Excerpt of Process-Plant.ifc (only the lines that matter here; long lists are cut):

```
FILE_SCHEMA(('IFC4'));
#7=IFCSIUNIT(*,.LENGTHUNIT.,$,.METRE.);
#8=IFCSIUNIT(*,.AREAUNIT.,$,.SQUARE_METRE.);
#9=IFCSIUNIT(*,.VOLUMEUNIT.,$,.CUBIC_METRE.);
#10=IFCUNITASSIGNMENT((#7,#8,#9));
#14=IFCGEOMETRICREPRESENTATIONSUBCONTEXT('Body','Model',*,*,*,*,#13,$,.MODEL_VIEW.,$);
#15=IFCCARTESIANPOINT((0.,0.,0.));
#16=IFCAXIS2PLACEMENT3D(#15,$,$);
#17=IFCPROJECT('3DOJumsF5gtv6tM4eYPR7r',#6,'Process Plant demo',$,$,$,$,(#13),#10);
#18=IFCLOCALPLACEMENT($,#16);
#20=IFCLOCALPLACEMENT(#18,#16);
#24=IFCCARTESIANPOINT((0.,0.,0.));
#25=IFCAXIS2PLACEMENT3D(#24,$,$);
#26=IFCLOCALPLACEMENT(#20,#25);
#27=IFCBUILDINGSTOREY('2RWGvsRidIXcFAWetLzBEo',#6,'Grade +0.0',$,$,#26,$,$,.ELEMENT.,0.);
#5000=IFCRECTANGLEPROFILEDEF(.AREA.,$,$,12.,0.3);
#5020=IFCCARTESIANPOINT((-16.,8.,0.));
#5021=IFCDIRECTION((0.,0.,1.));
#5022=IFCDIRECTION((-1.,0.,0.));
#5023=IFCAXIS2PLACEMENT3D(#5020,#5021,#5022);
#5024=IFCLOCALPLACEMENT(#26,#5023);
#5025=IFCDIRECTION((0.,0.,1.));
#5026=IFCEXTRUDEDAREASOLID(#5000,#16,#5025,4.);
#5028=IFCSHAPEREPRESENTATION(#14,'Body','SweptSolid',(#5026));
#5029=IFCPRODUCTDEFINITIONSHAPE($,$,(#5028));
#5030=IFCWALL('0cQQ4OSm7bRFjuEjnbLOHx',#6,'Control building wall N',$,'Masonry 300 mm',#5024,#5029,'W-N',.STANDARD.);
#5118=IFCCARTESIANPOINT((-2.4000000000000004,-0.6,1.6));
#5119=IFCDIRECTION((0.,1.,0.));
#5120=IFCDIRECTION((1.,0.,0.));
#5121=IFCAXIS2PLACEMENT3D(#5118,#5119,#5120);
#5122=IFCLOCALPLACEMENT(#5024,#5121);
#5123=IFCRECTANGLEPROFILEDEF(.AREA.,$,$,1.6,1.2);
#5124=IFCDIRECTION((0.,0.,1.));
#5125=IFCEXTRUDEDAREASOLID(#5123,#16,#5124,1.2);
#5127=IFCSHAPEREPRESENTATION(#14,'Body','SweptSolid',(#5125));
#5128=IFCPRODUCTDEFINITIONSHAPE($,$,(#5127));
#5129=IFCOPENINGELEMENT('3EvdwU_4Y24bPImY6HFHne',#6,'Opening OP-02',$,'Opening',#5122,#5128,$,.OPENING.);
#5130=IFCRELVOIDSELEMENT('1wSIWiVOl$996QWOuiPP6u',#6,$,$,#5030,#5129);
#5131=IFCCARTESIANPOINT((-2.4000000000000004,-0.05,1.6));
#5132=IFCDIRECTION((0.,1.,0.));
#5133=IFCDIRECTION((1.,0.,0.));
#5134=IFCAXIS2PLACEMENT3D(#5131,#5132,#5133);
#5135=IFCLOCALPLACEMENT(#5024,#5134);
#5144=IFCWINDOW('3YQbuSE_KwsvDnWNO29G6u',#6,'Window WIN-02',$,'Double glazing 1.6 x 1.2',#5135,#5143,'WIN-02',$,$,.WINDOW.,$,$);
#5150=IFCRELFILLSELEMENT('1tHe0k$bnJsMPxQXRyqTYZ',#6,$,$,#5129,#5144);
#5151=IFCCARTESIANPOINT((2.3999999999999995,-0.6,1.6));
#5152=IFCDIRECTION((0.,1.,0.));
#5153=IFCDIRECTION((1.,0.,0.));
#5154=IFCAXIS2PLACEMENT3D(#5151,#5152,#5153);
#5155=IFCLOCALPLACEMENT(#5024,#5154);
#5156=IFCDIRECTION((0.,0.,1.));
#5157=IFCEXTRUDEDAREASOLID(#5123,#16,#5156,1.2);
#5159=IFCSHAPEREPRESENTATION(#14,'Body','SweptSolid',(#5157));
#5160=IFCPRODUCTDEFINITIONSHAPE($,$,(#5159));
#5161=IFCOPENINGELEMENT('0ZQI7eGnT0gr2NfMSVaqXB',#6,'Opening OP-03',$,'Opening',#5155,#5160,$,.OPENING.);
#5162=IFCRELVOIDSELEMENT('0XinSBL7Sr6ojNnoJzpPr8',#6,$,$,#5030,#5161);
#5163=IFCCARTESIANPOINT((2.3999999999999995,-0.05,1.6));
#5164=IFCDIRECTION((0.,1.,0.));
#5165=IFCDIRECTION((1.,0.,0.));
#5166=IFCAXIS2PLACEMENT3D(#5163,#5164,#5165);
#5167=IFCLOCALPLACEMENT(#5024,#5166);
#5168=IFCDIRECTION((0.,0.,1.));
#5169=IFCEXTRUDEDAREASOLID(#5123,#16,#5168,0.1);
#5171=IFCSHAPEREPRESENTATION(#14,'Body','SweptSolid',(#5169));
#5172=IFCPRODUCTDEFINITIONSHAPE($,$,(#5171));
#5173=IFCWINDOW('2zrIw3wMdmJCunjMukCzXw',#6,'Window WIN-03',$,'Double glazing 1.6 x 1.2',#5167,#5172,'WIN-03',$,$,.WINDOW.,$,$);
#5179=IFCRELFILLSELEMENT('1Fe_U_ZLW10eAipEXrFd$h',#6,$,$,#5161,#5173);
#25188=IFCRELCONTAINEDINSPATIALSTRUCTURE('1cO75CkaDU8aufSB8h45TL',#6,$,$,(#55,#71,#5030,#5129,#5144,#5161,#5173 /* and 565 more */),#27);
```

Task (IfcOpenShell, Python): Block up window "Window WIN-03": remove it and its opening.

```python
import ifcopenshell
import ifcopenshell.api.feature
import ifcopenshell.api.root
import ifcopenshell.geom
import ifcopenshell.util.shape

model = ifcopenshell.open("Process-Plant.ifc")
settings = ifcopenshell.geom.settings()


def volume(element):
    """Net volume in cubic metres, openings subtracted."""
    shape = ifcopenshell.geom.create_shape(settings, element)
    return ifcopenshell.util.shape.get_volume(shape.geometry)


window = model.by_guid("2zrIw3wMdmJCunjMukCzXw")
opening = window.FillsVoids[0].RelatingOpeningElement
wall = opening.VoidsElements[0].RelatingBuildingElement
before = volume(wall)

ifcopenshell.api.root.remove_product(model, product=window)
ifcopenshell.api.feature.remove_feature(model, feature=opening)

after = volume(wall)

print(f"wall volume {before:.3f} -> {after:.3f} m3")

model.write("Process-Plant-out.ifc")
```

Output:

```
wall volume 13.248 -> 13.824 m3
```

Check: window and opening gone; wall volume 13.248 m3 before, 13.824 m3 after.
